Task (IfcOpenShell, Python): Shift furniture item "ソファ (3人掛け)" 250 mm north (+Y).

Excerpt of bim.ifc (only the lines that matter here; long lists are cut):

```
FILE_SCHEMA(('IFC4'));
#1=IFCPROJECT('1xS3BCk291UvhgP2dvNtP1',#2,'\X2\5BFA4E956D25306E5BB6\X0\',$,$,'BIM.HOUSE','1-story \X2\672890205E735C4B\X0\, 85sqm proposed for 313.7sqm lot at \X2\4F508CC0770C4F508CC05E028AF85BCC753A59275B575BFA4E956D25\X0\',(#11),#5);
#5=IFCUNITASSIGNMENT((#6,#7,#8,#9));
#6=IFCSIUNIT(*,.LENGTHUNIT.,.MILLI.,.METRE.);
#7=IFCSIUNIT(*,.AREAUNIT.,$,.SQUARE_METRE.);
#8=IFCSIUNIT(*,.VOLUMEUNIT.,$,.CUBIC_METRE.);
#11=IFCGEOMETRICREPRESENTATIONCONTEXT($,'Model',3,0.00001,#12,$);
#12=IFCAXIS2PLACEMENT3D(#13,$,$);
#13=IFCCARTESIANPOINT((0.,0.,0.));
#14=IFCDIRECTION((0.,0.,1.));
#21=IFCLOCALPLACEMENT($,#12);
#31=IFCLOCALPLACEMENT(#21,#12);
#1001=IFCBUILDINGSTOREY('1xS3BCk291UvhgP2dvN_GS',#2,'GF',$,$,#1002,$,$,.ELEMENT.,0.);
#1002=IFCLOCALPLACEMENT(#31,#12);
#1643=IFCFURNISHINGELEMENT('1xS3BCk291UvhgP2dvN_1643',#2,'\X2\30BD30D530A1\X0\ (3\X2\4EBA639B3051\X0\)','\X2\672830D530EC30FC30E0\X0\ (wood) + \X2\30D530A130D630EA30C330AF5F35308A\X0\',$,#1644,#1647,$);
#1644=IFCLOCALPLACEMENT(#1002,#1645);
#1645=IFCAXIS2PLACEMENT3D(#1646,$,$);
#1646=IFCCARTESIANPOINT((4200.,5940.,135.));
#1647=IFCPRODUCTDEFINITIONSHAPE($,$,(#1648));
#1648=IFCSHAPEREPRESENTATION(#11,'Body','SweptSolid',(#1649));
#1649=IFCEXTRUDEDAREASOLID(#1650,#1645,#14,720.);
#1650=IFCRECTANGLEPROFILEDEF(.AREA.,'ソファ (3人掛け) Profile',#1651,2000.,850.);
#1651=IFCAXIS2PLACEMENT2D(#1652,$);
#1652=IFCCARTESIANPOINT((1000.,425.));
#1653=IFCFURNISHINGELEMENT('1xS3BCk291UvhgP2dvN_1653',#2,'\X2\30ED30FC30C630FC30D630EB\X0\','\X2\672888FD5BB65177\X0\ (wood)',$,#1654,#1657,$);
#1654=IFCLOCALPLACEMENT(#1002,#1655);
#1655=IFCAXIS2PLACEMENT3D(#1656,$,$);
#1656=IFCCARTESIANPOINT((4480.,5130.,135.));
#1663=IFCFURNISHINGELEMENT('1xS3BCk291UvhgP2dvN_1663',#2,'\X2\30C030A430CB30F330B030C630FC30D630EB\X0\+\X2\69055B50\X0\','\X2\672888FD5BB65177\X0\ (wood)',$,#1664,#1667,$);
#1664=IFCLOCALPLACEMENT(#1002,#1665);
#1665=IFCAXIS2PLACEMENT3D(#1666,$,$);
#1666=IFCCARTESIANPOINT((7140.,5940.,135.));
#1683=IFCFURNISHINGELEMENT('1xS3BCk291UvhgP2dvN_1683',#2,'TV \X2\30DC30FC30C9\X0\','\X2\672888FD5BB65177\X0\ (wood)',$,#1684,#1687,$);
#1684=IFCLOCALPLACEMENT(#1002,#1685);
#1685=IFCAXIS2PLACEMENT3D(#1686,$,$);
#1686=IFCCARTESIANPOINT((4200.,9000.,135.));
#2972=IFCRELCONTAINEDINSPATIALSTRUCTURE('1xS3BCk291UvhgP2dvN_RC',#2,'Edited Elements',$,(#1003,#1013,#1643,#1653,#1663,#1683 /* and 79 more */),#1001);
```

```python
import ifcopenshell
import ifcopenshell.api.geometry
import ifcopenshell.util.placement
import ifcopenshell.util.unit

model = ifcopenshell.open("bim.ifc")
unit_scale = ifcopenshell.util.unit.calculate_unit_scale(model)

item = model.by_guid("1xS3BCk291UvhgP2dvN_1643")
matrix = ifcopenshell.util.placement.get_local_placement(item.ObjectPlacement)
matrix[1, 3] += 0.25 / unit_scale
ifcopenshell.api.geometry.edit_object_placement(model, product=item, matrix=matrix, is_si=False)

print(ifcopenshell.util.placement.get_local_placement(item.ObjectPlacement).round(3) + 0.0)

model.write("bim-out.ifc")
```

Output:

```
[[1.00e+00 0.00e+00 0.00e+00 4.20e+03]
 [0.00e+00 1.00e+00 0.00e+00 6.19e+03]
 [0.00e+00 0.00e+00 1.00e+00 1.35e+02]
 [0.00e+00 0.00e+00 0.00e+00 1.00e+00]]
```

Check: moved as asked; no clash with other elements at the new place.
